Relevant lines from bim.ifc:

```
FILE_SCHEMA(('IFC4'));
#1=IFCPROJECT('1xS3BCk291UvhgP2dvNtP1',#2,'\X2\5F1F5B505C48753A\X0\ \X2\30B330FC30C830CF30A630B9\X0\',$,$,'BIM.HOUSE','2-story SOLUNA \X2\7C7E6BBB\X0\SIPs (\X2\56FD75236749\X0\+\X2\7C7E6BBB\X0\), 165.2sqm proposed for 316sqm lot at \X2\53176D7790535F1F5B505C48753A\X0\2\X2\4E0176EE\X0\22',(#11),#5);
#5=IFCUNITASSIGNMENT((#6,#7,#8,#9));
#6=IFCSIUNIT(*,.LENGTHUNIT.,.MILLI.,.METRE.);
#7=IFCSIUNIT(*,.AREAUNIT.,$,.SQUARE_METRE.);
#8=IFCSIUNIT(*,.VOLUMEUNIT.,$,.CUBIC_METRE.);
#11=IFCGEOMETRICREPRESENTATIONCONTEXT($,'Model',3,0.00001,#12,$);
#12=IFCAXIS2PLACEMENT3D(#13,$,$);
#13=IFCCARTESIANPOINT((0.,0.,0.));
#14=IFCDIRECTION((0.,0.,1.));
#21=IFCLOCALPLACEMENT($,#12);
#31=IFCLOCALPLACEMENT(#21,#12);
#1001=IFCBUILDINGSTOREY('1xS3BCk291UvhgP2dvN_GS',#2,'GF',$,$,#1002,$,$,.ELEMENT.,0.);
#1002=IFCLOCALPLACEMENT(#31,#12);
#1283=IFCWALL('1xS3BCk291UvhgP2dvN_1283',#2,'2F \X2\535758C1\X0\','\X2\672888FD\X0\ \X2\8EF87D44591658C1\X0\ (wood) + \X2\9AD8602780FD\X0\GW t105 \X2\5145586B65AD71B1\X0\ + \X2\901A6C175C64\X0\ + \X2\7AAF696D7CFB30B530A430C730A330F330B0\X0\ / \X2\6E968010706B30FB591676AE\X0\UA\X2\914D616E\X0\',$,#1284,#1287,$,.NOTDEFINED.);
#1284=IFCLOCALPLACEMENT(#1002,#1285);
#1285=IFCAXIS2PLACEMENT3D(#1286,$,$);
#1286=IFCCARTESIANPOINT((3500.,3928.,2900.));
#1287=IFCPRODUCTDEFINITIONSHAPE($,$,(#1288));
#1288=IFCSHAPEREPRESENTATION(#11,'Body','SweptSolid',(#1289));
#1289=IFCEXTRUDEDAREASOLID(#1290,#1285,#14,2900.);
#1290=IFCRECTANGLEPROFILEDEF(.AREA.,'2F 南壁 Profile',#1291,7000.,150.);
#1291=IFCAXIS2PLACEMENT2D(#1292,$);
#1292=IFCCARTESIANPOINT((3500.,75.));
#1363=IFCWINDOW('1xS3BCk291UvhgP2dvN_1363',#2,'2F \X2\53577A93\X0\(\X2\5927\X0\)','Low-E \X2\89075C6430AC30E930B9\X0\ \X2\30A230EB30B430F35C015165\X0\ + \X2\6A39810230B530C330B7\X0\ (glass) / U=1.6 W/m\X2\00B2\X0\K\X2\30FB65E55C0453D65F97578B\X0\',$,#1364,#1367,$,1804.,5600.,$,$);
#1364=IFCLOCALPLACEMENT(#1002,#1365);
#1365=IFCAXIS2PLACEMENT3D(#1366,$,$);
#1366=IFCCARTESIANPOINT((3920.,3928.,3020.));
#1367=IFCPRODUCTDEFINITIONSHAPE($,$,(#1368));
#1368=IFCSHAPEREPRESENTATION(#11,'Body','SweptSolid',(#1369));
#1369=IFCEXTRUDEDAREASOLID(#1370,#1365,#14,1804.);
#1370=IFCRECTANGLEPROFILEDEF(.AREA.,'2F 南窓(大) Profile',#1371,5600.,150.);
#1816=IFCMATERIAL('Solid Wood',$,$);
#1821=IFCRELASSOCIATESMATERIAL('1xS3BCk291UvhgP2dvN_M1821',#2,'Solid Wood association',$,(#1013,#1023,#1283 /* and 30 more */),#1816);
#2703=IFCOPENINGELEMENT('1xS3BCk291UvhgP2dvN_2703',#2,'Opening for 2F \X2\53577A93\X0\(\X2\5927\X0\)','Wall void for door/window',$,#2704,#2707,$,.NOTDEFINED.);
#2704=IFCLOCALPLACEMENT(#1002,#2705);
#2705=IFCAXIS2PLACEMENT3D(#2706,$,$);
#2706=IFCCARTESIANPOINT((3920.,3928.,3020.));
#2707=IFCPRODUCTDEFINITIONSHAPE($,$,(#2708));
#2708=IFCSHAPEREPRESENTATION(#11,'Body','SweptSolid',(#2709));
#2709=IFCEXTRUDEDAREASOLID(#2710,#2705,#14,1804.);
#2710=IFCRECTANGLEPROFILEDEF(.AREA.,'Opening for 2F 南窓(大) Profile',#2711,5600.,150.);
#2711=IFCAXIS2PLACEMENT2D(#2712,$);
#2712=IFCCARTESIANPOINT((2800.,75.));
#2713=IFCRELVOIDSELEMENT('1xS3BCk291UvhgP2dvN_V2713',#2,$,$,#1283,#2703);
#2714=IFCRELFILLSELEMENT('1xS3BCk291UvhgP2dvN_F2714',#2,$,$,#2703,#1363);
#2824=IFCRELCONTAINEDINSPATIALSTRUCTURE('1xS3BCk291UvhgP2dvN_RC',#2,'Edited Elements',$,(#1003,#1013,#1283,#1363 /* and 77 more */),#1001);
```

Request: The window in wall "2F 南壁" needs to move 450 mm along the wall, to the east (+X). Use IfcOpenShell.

```python
import ifcopenshell
import ifcopenshell.api.geometry
import ifcopenshell.util.placement

model = ifcopenshell.open("bim.ifc")

window = model.by_guid("1xS3BCk291UvhgP2dvN_1363")
opening = window.FillsVoids[0].RelatingOpeningElement
wall = opening.VoidsElements[0].RelatingBuildingElement

wall_matrix = ifcopenshell.util.placement.get_local_placement(wall.ObjectPlacement)
shift = wall_matrix[:3, 0] * 450.0
before = ifcopenshell.util.placement.get_local_placement(window.ObjectPlacement)[:3, 3].copy()

# The window is not placed relative to its opening, so move both.
for product in (opening, window):
    matrix = ifcopenshell.util.placement.get_local_placement(product.ObjectPlacement)
    matrix[:3, 3] += shift
    ifcopenshell.api.geometry.edit_object_placement(model, product=product, matrix=matrix, is_si=False)

after = ifcopenshell.util.placement.get_local_placement(window.ObjectPlacement)[:3, 3]
print("window moved by", (after - before).round(3) + 0.0)

model.write("bim_v2.ifc")
```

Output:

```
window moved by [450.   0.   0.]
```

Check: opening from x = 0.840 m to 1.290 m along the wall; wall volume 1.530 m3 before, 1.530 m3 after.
